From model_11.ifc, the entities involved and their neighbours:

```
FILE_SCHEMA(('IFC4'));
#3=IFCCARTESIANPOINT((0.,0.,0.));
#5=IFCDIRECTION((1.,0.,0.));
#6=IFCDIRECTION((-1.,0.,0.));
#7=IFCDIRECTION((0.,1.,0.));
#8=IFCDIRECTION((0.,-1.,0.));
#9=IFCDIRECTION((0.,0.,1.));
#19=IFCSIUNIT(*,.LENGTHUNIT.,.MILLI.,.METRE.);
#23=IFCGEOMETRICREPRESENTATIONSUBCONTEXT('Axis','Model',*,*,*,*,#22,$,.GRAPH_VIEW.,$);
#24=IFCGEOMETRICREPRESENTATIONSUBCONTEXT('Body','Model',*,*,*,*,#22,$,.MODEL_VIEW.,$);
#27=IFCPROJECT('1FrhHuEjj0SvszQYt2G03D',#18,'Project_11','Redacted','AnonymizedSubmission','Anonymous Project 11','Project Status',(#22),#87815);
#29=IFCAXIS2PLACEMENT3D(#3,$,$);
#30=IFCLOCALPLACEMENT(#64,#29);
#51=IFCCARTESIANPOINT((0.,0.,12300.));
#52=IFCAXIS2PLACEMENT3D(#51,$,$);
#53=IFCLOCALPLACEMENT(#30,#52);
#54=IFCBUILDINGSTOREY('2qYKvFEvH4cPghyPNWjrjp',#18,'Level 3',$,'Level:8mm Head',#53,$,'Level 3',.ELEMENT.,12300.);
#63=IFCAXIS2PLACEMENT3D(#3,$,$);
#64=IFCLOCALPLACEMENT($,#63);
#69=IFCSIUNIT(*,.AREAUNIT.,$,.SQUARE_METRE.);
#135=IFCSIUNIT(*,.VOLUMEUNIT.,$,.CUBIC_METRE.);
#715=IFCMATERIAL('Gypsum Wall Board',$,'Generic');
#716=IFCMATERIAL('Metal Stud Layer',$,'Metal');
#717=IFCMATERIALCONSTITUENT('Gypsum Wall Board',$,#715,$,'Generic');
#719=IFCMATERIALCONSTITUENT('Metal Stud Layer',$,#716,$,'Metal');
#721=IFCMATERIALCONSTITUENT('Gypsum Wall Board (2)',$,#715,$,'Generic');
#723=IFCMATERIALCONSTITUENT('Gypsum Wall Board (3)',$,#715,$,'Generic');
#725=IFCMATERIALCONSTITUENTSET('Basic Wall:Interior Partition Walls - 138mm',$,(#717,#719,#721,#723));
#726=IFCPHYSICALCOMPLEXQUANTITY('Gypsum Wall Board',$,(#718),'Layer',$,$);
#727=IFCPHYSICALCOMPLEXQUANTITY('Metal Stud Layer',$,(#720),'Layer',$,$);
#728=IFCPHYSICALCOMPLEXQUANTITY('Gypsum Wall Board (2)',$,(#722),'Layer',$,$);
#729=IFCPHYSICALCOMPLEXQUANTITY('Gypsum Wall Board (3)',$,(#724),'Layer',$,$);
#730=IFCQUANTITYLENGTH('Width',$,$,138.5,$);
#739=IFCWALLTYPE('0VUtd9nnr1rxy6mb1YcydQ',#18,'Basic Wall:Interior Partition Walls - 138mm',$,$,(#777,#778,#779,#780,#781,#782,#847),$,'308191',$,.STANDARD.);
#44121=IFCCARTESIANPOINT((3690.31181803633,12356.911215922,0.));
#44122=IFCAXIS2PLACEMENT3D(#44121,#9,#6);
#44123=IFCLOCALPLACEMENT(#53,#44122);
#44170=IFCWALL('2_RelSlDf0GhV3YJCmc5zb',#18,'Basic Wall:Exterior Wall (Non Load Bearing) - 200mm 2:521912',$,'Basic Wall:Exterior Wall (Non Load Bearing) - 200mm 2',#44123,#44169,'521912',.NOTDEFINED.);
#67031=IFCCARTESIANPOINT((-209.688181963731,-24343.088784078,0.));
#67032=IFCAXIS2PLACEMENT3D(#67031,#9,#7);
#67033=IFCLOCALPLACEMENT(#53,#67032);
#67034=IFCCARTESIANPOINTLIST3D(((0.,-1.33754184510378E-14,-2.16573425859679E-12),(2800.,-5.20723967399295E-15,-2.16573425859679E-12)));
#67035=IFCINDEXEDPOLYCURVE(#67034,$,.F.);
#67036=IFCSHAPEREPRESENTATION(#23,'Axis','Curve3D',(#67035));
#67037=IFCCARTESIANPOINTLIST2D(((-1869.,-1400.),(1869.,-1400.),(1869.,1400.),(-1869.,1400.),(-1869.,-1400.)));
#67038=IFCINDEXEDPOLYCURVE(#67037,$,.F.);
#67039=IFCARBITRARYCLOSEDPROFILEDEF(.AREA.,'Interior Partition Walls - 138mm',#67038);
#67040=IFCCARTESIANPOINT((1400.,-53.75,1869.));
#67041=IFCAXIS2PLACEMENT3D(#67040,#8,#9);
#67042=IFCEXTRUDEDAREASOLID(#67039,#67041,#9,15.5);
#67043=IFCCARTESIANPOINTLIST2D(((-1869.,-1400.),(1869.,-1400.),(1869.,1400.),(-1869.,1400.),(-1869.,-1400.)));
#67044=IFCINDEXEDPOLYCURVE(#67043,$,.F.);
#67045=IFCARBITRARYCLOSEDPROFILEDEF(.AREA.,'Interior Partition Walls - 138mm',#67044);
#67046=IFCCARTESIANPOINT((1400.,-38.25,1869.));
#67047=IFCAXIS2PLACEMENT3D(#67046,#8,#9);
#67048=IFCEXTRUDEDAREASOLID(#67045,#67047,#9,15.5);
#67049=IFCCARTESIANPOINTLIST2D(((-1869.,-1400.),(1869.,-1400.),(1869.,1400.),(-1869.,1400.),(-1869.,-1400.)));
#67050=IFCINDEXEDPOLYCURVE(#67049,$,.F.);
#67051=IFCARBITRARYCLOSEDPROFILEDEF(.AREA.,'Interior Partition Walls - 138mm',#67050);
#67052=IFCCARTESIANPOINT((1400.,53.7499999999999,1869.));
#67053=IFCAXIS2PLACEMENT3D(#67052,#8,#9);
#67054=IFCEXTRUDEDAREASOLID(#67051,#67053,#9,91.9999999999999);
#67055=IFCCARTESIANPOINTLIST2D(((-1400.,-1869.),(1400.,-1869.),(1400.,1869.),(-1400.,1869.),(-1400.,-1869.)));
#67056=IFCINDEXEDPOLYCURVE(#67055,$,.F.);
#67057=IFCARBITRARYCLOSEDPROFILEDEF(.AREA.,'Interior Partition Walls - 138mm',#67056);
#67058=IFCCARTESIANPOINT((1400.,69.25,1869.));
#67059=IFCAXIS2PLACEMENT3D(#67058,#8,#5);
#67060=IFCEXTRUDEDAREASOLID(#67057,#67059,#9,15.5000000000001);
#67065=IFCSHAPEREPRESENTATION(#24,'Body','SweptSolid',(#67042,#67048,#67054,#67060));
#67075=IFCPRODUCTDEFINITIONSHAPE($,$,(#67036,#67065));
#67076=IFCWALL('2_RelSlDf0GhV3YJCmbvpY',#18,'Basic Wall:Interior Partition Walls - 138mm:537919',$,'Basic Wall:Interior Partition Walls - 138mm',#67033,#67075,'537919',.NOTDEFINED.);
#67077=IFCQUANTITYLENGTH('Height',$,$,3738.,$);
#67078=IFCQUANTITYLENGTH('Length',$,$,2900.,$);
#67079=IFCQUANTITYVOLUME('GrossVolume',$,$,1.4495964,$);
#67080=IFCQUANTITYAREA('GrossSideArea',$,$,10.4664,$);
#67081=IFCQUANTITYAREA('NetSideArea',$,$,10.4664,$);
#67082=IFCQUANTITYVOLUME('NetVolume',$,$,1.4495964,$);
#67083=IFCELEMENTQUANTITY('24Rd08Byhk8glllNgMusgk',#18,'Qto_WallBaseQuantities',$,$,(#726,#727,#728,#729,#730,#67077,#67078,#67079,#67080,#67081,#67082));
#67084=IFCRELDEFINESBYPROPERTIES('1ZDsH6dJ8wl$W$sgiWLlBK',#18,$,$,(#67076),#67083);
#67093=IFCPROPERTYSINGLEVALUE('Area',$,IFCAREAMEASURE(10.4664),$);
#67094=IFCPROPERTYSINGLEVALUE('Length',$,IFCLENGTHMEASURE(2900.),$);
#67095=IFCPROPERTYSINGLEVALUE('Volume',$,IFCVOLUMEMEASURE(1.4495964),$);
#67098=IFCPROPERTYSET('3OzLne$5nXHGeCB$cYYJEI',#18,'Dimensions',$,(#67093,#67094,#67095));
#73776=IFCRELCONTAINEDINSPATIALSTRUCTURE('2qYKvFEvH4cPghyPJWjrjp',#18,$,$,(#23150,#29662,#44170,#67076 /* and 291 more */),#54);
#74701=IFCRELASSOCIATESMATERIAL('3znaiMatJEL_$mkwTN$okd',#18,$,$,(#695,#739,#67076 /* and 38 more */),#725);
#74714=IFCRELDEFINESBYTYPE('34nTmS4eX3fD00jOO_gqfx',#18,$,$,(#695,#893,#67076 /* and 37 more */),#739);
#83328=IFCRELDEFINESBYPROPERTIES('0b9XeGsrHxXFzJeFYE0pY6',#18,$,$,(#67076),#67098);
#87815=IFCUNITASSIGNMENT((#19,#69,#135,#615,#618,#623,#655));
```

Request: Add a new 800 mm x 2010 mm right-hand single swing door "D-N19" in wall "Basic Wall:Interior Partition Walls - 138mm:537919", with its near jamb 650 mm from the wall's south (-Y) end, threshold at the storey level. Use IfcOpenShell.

```python
import numpy as np
import ifcopenshell
import ifcopenshell.api.feature
import ifcopenshell.api.geometry
import ifcopenshell.api.pset
import ifcopenshell.api.root
import ifcopenshell.api.spatial
import ifcopenshell.geom
import ifcopenshell.util.element
import ifcopenshell.util.placement
import ifcopenshell.util.representation
import ifcopenshell.util.shape
import ifcopenshell.util.unit

model = ifcopenshell.open("model_11.ifc")
unit_scale = ifcopenshell.util.unit.calculate_unit_scale(model)
area_scale = ifcopenshell.util.unit.calculate_unit_scale(model, "AREAUNIT")
volume_scale = ifcopenshell.util.unit.calculate_unit_scale(model, "VOLUMEUNIT")
settings = ifcopenshell.geom.settings()


def volume(element):
    """Net volume in cubic metres, openings subtracted."""
    shape = ifcopenshell.geom.create_shape(settings, element)
    return ifcopenshell.util.shape.get_volume(shape.geometry)


wall = model.by_guid("2_RelSlDf0GhV3YJCmbvpY")
storey = ifcopenshell.util.element.get_container(wall, ifc_class="IfcBuildingStorey")
context = ifcopenshell.util.representation.get_context(model, "Model", "Body", "MODEL_VIEW")
before = volume(wall)

width, height, from_end, sill = 0.8, 2.01, 0.65, 0.0  # metres

# The wall runs along its own X axis, and the end named is its -X end.
wall_shape = ifcopenshell.geom.create_shape(settings, wall)
x, y, z = ifcopenshell.util.shape.get_vertices(wall_shape.geometry).T
start = x.min() + from_end
face, thickness = float(y.min()), float(y.max() - y.min())
wall_matrix = ifcopenshell.util.placement.get_local_placement(wall.ObjectPlacement)
level = ifcopenshell.util.placement.get_local_placement(storey.ObjectPlacement)[2, 3]


def in_wall(x, y):
    """Placement at x, y metres in the wall's axes, at sill height."""
    matrix = wall_matrix.copy()
    matrix[:, 3] = wall_matrix @ np.array([x / unit_scale, y / unit_scale, 0.0, 1.0])
    matrix[2, 3] = level + sill / unit_scale
    return matrix


# Opening: a box that overshoots both wall faces by 50 mm.
opening = ifcopenshell.api.root.create_entity(model, ifc_class="IfcOpeningElement", predefined_type="OPENING")
box = ifcopenshell.api.geometry.add_wall_representation(
    model, context=context, length=width, height=height, thickness=thickness + 0.1
)
ifcopenshell.api.geometry.assign_representation(model, product=opening, representation=box)
ifcopenshell.api.geometry.edit_object_placement(model, product=opening, matrix=in_wall(start, face - 0.05), is_si=False)
ifcopenshell.api.feature.add_feature(model, feature=opening, element=wall)

door = ifcopenshell.api.root.create_entity(model, ifc_class="IfcDoor", name="D-N19", predefined_type="DOOR")
door.OverallWidth, door.OverallHeight = width / unit_scale, height / unit_scale
door.OperationType = "SINGLE_SWING_RIGHT"
body = ifcopenshell.api.geometry.add_door_representation(
    model,
    context=context,
    overall_width=door.OverallWidth,
    overall_height=door.OverallHeight,
    operation_type="SINGLE_SWING_RIGHT",
    lining_properties={"LiningDepth": thickness / unit_scale, "ThresholdDepth": thickness / unit_scale},
)
ifcopenshell.api.geometry.assign_representation(model, product=door, representation=body)
ifcopenshell.api.spatial.assign_container(model, products=[door], relating_structure=storey)
ifcopenshell.api.feature.add_filling(model, opening=opening, element=door)

# The lining spans the wall, so the door starts at the wall face.
ifcopenshell.api.geometry.edit_object_placement(model, product=door, matrix=in_wall(start, face), is_si=False)

after = volume(wall)

# Update the wall's stored quantities.
qto = model.by_id(ifcopenshell.util.element.get_pset(wall, "Qto_WallBaseQuantities", should_inherit=False)["id"])
ifcopenshell.api.pset.edit_qto(model, qto=qto, properties={
    "NetSideArea": after / thickness / area_scale,
    "NetVolume": after / volume_scale,
})
pset = model.by_id(ifcopenshell.util.element.get_pset(wall, "Dimensions", should_inherit=False)["id"])
ifcopenshell.api.pset.edit_pset(model, pset=pset, properties={
    "Area": model.create_entity("IfcAreaMeasure", after / thickness / area_scale),
    "Volume": model.create_entity("IfcVolumeMeasure", after / volume_scale),
})

print(f"wall volume {before:.3f} -> {after:.3f} m3")

model.write("model_11_v2.ifc")
```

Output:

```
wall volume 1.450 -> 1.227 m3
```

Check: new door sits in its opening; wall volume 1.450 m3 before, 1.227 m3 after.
